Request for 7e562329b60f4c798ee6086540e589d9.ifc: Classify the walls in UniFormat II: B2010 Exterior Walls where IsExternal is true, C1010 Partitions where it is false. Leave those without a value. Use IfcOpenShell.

First a look at what the model holds.

```python
import ifcopenshell
import ifcopenshell.util.element

model = ifcopenshell.open("7e562329b60f4c798ee6086540e589d9.ifc")
print(model.schema)
print("classifications:", [c.Name for c in model.by_type("IfcClassification")])
values = [ifcopenshell.util.element.get_pset(e, "Pset_WallCommon", "IsExternal") for e in model.by_type("IfcWall")]
for value in (True, False, None):
    print("IsExternal", value, values.count(value))
```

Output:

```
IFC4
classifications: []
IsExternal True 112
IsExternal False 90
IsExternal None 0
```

```python
import ifcopenshell
import ifcopenshell.api.classification
import ifcopenshell.util.element

model = ifcopenshell.open("7e562329b60f4c798ee6086540e589d9.ifc")

system = ifcopenshell.api.classification.add_classification(model, classification="UniFormat II")

walls = model.by_type("IfcWall")
external = {e: ifcopenshell.util.element.get_pset(e, "Pset_WallCommon", "IsExternal") for e in walls}
for flag, code, name in ((True, "B2010", "Exterior Walls"), (False, "C1010", "Partitions")):
    products = [e for e in walls if external[e] is flag]
    ifcopenshell.api.classification.add_reference(
        model, products=products, classification=system, identification=code, name=name
    )
    print(code, len(products))

model.write("7e562329b60f4c798ee6086540e589d9_updated.ifc")
```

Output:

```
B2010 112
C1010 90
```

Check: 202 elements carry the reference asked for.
